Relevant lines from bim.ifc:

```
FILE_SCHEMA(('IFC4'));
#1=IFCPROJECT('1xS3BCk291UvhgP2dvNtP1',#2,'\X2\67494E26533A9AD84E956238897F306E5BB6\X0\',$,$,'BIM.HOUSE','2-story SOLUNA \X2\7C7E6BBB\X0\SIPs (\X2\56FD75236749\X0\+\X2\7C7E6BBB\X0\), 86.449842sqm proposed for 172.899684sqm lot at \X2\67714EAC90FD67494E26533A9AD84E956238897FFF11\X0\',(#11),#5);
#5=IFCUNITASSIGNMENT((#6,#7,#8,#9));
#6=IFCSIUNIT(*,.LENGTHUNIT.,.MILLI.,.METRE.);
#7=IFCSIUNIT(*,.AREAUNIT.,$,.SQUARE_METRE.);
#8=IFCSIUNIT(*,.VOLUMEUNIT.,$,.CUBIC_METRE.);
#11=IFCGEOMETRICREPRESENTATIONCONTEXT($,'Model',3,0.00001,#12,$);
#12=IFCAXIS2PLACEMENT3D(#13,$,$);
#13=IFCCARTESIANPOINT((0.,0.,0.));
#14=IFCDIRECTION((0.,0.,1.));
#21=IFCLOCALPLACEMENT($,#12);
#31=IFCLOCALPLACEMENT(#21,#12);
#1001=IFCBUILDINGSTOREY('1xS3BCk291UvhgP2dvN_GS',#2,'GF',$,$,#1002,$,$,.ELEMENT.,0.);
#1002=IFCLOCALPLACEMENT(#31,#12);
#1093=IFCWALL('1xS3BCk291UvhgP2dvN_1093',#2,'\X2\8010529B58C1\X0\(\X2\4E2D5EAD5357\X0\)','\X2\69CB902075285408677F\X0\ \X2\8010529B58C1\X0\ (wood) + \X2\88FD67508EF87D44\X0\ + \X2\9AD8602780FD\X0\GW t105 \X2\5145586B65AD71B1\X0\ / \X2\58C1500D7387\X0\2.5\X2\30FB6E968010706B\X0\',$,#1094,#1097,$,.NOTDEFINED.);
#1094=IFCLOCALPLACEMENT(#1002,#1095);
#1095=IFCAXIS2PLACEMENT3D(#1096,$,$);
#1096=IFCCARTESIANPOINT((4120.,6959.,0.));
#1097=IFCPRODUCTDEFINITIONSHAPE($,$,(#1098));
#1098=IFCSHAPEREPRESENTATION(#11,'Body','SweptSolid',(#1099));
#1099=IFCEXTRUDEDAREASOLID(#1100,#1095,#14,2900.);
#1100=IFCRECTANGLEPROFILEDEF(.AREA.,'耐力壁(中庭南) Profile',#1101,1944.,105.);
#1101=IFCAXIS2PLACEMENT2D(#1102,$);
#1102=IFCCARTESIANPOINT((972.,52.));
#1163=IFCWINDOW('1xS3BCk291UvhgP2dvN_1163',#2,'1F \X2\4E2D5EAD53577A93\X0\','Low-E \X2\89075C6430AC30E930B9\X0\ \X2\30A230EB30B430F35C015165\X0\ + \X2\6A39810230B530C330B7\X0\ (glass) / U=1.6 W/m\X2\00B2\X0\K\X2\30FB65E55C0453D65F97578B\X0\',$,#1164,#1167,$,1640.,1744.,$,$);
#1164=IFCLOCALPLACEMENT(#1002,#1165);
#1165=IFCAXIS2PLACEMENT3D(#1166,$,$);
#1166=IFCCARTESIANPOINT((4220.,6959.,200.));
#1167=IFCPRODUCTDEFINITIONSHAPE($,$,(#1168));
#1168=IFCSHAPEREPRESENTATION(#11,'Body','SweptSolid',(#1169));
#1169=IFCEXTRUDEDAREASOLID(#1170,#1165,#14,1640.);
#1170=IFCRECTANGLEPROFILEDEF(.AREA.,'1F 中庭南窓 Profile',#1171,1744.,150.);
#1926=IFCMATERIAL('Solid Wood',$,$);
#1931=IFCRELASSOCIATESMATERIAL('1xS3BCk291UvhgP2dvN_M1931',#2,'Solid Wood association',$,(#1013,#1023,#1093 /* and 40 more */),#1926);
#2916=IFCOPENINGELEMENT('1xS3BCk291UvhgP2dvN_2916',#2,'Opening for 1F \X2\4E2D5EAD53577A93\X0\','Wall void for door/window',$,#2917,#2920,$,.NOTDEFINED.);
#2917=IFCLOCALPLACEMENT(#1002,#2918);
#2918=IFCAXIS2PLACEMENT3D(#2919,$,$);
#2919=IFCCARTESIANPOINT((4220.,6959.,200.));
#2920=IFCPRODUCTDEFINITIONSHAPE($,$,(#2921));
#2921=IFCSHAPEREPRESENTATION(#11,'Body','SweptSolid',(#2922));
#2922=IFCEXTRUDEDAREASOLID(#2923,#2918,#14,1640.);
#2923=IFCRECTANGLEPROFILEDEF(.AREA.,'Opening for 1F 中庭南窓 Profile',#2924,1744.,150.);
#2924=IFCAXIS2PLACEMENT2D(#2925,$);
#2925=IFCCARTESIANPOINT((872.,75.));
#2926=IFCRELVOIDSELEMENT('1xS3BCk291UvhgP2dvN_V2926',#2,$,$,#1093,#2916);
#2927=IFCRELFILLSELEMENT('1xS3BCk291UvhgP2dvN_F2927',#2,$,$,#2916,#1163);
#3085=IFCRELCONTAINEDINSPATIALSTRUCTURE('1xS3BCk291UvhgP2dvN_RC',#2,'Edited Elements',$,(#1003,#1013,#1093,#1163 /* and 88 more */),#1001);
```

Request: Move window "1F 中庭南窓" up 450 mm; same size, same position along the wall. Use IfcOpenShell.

```python
import numpy as np
import ifcopenshell
import ifcopenshell.api.geometry
import ifcopenshell.util.placement
import ifcopenshell.util.unit

model = ifcopenshell.open("bim.ifc")
unit_scale = ifcopenshell.util.unit.calculate_unit_scale(model)

window = model.by_id(1163)
opening = window.FillsVoids[0].RelatingOpeningElement
dz = 450.0

shift = np.array([0.0, 0.0, dz])
# The window is not placed relative to its opening, so move both.
for product in (opening, window):
    matrix = ifcopenshell.util.placement.get_local_placement(product.ObjectPlacement)
    matrix[:3, 3] += shift
    ifcopenshell.api.geometry.edit_object_placement(model, product=product, matrix=matrix, is_si=False)

print(f"moved by {dz * unit_scale:+.3f} m")

model.write("bim_v2.ifc")
```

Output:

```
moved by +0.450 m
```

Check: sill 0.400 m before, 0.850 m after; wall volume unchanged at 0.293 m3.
